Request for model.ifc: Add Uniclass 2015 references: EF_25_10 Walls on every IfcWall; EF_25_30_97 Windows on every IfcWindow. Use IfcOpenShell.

First a look at what the model holds.

```python
import ifcopenshell

model = ifcopenshell.open("model.ifc")
print(model.schema)
print("classifications:", [c.Name for c in model.by_type("IfcClassification")])
for ifc_class in ("IfcDoor", "IfcRoof", "IfcStair", "IfcWall", "IfcWindow"):
    print(ifc_class, len(model.by_type(ifc_class)))
```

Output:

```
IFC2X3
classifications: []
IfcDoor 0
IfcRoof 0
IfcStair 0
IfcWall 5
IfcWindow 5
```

```python
import ifcopenshell
import ifcopenshell.api.classification

model = ifcopenshell.open("model.ifc")

# IFC2X3 requires Source and Edition and has no link from the project to the system.
system = model.create_entity("IfcClassification", Source="NBS", Edition="2015", Name="Uniclass 2015")

codes = {
    "IfcWall": ("EF_25_10", "Walls"),
    "IfcWindow": ("EF_25_30_97", "Windows"),
}
for ifc_class, (code, name) in codes.items():
    products = model.by_type(ifc_class)
    ifcopenshell.api.classification.add_reference(
        model, products=products, classification=system, identification=code, name=name
    )
    print(code, len(products))

model.write("model_updated.ifc")
```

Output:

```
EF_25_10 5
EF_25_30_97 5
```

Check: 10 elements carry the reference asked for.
